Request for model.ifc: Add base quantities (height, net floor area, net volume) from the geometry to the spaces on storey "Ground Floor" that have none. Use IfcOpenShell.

First a look at what the model holds.

```python
import ifcopenshell
import ifcopenshell.util.element
import ifcopenshell.util.unit

model = ifcopenshell.open("model.ifc")
print(model.schema)
for unit_type in ("LENGTHUNIT", "AREAUNIT", "VOLUMEUNIT"):
    print(unit_type, ifcopenshell.util.unit.calculate_unit_scale(model, unit_type))
storey = next(s for s in model.by_type("IfcBuildingStorey") if s.Name == "Ground Floor")
spaces = [e for e in ifcopenshell.util.element.get_decomposition(storey) if e.is_a("IfcSpace")]
for e in sorted(spaces, key=lambda e: e.id()):
    print(e.id(), e.is_a(), e.Name, list(ifcopenshell.util.element.get_psets(e, qtos_only=True)), sep=" | ")
```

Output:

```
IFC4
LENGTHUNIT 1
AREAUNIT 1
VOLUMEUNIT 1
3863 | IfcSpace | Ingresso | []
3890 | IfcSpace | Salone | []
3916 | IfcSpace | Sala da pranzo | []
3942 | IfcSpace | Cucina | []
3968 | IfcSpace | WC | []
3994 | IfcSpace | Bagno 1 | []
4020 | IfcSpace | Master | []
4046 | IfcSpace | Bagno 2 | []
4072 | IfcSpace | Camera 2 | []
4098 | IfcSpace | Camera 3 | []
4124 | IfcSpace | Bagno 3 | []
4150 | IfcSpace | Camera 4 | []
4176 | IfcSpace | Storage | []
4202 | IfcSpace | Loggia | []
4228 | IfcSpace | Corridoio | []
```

```python
import ifcopenshell
import ifcopenshell.api.pset
import ifcopenshell.geom
import ifcopenshell.util.element
import ifcopenshell.util.shape
import ifcopenshell.util.unit

model = ifcopenshell.open("model.ifc")
unit_scale = ifcopenshell.util.unit.calculate_unit_scale(model)
area_scale = ifcopenshell.util.unit.calculate_unit_scale(model, "AREAUNIT")
volume_scale = ifcopenshell.util.unit.calculate_unit_scale(model, "VOLUMEUNIT")
settings = ifcopenshell.geom.settings()

storey = next(s for s in model.by_type("IfcBuildingStorey") if s.Name == "Ground Floor")
spaces = [e for e in ifcopenshell.util.element.get_decomposition(storey) if e.is_a("IfcSpace")]

for e in sorted(spaces, key=lambda e: e.id()):
    if ifcopenshell.util.element.get_psets(e, qtos_only=True, should_inherit=False):
        continue
    # Geometry comes back in metres, in the element's own axes.
    shape = ifcopenshell.geom.create_shape(settings, e)
    values = {
        "Height": ifcopenshell.util.shape.get_z(shape.geometry) / unit_scale,
        "NetFloorArea": ifcopenshell.util.shape.get_footprint_area(shape.geometry) / area_scale,
        "NetVolume": ifcopenshell.util.shape.get_volume(shape.geometry) / volume_scale,
    }
    qto = ifcopenshell.api.pset.add_qto(model, product=e, name="Qto_SpaceBaseQuantities")
    ifcopenshell.api.pset.edit_qto(model, qto=qto, properties=values)
    print(e.id(), {k: round(v, 3) for k, v in values.items()})

model.write("model_v2.ifc")
```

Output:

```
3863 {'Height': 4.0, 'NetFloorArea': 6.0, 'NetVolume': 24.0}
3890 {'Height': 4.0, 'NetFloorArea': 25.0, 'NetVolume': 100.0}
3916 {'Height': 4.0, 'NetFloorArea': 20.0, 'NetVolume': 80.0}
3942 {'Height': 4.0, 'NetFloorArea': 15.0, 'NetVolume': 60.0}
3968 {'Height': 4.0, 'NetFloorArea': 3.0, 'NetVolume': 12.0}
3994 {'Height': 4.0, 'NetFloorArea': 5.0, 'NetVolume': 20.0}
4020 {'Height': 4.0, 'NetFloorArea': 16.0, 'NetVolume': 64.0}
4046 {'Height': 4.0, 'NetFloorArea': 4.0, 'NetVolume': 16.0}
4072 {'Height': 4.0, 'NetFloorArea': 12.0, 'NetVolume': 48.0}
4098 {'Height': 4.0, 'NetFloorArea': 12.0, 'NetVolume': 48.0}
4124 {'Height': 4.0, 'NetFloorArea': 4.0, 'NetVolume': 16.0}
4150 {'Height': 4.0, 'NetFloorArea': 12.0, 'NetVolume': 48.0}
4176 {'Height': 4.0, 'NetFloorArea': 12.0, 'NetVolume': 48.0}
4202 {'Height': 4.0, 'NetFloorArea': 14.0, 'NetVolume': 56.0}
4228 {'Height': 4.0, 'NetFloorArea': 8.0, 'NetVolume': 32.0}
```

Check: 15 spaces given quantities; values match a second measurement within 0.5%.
